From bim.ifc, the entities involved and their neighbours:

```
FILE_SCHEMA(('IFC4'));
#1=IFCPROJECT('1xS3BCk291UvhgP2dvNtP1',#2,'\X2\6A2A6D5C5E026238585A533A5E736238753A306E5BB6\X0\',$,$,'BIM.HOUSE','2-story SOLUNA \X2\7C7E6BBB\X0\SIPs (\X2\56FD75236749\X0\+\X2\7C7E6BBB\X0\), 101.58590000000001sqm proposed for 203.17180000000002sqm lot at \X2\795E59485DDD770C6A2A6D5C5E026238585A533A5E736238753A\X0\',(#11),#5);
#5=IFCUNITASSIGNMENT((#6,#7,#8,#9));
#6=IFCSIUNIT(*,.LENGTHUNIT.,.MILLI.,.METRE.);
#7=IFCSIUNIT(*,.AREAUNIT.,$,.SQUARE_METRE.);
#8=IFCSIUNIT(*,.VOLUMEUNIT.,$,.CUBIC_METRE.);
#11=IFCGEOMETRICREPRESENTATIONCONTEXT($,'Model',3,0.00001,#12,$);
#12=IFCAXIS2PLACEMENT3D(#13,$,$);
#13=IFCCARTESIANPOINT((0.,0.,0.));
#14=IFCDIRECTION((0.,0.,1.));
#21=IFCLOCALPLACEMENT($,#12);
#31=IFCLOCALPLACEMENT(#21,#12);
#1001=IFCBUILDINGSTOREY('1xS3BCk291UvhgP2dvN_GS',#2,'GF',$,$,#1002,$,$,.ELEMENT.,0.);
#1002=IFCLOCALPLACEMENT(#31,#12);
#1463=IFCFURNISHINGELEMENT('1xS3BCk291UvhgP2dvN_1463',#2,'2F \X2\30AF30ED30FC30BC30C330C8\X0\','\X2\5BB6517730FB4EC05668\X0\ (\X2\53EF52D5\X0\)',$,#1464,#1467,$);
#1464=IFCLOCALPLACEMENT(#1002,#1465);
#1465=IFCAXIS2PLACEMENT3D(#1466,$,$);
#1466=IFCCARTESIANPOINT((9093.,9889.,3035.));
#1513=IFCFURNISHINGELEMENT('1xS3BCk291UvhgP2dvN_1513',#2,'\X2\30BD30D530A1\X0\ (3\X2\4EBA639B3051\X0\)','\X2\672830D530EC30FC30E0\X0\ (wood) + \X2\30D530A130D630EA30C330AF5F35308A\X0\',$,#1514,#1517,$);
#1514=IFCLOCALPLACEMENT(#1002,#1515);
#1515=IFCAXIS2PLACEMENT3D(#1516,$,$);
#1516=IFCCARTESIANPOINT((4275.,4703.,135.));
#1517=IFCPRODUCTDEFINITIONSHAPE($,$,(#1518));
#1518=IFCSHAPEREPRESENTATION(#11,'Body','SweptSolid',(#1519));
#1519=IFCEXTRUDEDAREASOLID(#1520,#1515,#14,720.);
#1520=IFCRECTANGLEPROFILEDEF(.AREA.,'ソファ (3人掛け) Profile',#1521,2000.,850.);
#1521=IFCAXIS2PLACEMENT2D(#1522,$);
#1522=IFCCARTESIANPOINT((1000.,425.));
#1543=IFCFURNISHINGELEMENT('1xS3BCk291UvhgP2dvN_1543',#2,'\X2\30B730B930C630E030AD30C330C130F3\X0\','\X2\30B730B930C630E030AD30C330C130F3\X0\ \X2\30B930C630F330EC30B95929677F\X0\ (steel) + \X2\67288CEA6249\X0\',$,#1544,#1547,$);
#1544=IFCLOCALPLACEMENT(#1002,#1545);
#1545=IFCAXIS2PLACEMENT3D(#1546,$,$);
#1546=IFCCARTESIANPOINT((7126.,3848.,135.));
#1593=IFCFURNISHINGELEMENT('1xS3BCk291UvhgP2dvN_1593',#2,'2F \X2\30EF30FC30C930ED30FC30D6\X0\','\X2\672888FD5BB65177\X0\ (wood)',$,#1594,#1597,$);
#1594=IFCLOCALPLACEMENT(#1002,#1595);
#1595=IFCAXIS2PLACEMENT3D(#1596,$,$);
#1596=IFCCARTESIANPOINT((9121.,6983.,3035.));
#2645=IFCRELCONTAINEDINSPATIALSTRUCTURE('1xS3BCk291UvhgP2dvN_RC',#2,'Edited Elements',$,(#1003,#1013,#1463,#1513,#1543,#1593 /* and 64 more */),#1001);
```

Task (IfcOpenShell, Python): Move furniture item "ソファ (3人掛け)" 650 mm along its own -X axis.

```python
import ifcopenshell
import ifcopenshell.api.geometry
import ifcopenshell.util.placement
import ifcopenshell.util.unit

model = ifcopenshell.open("bim.ifc")
unit_scale = ifcopenshell.util.unit.calculate_unit_scale(model)

item = model.by_guid("1xS3BCk291UvhgP2dvN_1513")
matrix = ifcopenshell.util.placement.get_local_placement(item.ObjectPlacement)
matrix[:3, 3] -= matrix[:3, 0] * 0.65 / unit_scale
ifcopenshell.api.geometry.edit_object_placement(model, product=item, matrix=matrix, is_si=False)

print(ifcopenshell.util.placement.get_local_placement(item.ObjectPlacement).round(3) + 0.0)

model.write("bim-out.ifc")
```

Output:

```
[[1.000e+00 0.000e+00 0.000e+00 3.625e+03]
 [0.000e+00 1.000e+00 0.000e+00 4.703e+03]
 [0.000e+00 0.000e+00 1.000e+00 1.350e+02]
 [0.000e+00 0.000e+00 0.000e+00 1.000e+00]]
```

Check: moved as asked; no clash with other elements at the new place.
